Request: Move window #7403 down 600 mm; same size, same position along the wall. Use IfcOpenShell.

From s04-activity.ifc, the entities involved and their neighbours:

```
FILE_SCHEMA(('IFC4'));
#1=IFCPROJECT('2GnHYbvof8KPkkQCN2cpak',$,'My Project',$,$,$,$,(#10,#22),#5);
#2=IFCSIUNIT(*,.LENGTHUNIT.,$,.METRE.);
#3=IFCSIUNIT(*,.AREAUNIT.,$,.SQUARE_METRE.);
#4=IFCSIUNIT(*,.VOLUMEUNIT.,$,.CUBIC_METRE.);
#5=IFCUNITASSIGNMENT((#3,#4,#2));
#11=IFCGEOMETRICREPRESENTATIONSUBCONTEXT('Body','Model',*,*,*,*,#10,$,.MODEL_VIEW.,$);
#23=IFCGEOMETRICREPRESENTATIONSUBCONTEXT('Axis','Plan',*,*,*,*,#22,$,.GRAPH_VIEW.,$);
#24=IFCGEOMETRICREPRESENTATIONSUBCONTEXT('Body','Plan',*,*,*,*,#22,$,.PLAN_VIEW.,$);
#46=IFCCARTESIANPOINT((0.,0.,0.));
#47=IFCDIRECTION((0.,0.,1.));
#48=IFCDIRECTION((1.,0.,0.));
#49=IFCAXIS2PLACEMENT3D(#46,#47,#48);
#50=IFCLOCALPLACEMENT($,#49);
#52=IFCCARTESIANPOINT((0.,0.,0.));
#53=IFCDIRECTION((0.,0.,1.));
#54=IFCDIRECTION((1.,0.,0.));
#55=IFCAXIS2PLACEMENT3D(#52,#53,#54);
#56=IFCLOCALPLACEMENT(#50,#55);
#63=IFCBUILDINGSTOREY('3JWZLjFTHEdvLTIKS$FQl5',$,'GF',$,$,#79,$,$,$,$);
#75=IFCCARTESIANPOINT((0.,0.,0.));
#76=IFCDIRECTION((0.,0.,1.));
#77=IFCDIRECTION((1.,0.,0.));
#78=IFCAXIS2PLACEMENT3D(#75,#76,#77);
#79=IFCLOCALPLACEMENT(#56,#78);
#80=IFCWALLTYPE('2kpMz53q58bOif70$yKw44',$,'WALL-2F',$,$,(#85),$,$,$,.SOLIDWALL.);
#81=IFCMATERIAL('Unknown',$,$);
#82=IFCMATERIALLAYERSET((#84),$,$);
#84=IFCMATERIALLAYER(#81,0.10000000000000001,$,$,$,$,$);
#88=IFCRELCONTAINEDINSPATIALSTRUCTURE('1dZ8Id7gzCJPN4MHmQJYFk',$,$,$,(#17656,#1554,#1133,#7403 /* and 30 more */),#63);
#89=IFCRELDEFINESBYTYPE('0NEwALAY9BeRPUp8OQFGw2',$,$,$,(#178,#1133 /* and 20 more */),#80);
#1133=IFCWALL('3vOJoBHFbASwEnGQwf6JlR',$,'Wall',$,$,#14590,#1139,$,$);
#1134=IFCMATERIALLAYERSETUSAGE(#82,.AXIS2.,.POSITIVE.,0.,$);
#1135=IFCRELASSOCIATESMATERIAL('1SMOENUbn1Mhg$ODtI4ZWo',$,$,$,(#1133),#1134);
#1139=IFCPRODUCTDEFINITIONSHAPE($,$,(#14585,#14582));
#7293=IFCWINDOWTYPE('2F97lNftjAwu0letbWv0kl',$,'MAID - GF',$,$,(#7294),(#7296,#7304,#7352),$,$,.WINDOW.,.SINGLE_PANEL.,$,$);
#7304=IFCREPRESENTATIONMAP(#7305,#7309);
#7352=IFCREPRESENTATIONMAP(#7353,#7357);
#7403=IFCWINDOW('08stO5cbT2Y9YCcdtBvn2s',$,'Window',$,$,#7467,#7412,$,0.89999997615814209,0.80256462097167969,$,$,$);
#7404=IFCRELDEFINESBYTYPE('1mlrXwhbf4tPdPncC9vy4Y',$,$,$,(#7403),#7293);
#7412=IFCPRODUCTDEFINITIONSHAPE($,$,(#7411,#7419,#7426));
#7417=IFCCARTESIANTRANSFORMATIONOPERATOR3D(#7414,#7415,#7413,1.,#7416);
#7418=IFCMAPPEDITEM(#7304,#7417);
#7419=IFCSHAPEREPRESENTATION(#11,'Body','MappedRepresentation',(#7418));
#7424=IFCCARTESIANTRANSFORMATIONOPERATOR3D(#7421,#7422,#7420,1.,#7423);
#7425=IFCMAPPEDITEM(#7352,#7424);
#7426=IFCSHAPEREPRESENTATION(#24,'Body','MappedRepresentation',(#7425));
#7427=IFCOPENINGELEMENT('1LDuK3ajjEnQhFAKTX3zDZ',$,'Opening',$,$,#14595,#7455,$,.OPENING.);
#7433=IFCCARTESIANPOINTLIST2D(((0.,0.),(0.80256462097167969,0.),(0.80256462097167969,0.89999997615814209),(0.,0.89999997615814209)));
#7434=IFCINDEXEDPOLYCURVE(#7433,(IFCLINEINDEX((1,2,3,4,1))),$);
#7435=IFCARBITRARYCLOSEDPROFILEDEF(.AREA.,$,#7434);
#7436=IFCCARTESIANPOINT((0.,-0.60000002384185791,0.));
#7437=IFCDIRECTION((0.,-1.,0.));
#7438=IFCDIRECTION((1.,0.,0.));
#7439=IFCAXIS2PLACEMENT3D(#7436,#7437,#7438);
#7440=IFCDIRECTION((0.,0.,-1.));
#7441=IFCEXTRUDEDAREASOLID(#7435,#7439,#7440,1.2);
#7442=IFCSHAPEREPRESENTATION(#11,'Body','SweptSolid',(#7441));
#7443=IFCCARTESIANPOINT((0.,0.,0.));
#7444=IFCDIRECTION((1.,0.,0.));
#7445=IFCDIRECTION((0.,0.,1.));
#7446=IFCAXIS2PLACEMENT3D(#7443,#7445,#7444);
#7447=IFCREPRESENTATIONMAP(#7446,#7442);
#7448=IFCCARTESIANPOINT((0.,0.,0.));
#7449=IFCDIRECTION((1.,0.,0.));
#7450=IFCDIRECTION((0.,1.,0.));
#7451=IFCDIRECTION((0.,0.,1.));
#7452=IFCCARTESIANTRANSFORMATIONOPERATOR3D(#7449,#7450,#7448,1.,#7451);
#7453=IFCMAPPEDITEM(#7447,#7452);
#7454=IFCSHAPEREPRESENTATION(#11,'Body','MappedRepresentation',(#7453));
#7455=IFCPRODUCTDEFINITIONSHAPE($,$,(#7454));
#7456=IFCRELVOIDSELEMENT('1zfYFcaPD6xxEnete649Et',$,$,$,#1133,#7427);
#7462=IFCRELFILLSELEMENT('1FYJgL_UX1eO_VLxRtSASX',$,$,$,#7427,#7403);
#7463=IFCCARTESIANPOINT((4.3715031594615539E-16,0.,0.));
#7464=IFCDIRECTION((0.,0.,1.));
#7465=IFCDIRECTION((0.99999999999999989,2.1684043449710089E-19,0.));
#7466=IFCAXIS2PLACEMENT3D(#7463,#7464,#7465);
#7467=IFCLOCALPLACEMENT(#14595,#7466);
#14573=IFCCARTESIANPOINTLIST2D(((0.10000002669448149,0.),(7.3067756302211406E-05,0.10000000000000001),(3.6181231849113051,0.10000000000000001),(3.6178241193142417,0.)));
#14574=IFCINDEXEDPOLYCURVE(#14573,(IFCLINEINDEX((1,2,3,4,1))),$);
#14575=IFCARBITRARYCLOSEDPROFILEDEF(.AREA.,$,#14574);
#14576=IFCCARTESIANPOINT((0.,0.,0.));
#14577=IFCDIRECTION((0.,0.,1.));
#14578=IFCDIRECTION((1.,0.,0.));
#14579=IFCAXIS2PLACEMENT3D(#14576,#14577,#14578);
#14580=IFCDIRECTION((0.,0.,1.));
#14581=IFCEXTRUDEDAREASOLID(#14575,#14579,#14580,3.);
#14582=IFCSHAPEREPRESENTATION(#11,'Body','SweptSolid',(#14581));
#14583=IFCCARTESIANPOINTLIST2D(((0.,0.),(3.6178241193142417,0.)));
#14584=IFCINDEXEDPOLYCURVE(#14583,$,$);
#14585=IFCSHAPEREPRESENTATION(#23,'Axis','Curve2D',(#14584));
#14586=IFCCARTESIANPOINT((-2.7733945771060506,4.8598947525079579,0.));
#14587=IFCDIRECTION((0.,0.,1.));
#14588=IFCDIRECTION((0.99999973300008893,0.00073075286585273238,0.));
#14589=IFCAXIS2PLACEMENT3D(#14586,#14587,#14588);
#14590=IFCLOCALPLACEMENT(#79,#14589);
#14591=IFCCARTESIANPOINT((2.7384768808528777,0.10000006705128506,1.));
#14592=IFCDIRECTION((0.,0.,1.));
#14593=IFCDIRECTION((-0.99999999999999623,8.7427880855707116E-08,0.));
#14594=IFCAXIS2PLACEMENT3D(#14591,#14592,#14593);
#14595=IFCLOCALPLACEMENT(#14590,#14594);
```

```python
import numpy as np
import ifcopenshell
import ifcopenshell.api.geometry
import ifcopenshell.util.placement
import ifcopenshell.util.unit

model = ifcopenshell.open("s04-activity.ifc")
unit_scale = ifcopenshell.util.unit.calculate_unit_scale(model)

window = model.by_guid("08stO5cbT2Y9YCcdtBvn2s")
opening = window.FillsVoids[0].RelatingOpeningElement
dz = -0.6

shift = np.array([0.0, 0.0, dz])
# The window is placed relative to its opening, so it follows when the opening moves.
matrix = ifcopenshell.util.placement.get_local_placement(opening.ObjectPlacement)
matrix[:3, 3] += shift
ifcopenshell.api.geometry.edit_object_placement(
    model, product=opening, matrix=matrix, is_si=False, should_transform_children=True
)

print(f"moved by {dz * unit_scale:+.3f} m")

model.write("s04-activity_rev.ifc")
```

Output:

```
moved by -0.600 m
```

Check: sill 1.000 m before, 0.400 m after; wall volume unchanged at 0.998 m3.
